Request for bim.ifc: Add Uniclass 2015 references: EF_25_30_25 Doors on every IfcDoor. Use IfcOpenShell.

First a look at what the model holds.

```python
import ifcopenshell

model = ifcopenshell.open("bim.ifc")
print(model.schema)
print("classifications:", [c.Name for c in model.by_type("IfcClassification")])
for ifc_class in ("IfcDoor", "IfcRoof", "IfcStair", "IfcWall", "IfcWindow"):
    print(ifc_class, len(model.by_type(ifc_class)))
```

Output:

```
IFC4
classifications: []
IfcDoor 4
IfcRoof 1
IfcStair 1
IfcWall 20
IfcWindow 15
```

```python
import ifcopenshell
import ifcopenshell.api.classification

model = ifcopenshell.open("bim.ifc")

system = ifcopenshell.api.classification.add_classification(model, classification="Uniclass 2015")

codes = {
    "IfcDoor": ("EF_25_30_25", "Doors"),
}
for ifc_class, (code, name) in codes.items():
    products = model.by_type(ifc_class)
    ifcopenshell.api.classification.add_reference(
        model, products=products, classification=system, identification=code, name=name
    )
    print(code, len(products))

model.write("bim_rev.ifc")
```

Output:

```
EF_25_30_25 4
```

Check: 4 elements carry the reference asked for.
